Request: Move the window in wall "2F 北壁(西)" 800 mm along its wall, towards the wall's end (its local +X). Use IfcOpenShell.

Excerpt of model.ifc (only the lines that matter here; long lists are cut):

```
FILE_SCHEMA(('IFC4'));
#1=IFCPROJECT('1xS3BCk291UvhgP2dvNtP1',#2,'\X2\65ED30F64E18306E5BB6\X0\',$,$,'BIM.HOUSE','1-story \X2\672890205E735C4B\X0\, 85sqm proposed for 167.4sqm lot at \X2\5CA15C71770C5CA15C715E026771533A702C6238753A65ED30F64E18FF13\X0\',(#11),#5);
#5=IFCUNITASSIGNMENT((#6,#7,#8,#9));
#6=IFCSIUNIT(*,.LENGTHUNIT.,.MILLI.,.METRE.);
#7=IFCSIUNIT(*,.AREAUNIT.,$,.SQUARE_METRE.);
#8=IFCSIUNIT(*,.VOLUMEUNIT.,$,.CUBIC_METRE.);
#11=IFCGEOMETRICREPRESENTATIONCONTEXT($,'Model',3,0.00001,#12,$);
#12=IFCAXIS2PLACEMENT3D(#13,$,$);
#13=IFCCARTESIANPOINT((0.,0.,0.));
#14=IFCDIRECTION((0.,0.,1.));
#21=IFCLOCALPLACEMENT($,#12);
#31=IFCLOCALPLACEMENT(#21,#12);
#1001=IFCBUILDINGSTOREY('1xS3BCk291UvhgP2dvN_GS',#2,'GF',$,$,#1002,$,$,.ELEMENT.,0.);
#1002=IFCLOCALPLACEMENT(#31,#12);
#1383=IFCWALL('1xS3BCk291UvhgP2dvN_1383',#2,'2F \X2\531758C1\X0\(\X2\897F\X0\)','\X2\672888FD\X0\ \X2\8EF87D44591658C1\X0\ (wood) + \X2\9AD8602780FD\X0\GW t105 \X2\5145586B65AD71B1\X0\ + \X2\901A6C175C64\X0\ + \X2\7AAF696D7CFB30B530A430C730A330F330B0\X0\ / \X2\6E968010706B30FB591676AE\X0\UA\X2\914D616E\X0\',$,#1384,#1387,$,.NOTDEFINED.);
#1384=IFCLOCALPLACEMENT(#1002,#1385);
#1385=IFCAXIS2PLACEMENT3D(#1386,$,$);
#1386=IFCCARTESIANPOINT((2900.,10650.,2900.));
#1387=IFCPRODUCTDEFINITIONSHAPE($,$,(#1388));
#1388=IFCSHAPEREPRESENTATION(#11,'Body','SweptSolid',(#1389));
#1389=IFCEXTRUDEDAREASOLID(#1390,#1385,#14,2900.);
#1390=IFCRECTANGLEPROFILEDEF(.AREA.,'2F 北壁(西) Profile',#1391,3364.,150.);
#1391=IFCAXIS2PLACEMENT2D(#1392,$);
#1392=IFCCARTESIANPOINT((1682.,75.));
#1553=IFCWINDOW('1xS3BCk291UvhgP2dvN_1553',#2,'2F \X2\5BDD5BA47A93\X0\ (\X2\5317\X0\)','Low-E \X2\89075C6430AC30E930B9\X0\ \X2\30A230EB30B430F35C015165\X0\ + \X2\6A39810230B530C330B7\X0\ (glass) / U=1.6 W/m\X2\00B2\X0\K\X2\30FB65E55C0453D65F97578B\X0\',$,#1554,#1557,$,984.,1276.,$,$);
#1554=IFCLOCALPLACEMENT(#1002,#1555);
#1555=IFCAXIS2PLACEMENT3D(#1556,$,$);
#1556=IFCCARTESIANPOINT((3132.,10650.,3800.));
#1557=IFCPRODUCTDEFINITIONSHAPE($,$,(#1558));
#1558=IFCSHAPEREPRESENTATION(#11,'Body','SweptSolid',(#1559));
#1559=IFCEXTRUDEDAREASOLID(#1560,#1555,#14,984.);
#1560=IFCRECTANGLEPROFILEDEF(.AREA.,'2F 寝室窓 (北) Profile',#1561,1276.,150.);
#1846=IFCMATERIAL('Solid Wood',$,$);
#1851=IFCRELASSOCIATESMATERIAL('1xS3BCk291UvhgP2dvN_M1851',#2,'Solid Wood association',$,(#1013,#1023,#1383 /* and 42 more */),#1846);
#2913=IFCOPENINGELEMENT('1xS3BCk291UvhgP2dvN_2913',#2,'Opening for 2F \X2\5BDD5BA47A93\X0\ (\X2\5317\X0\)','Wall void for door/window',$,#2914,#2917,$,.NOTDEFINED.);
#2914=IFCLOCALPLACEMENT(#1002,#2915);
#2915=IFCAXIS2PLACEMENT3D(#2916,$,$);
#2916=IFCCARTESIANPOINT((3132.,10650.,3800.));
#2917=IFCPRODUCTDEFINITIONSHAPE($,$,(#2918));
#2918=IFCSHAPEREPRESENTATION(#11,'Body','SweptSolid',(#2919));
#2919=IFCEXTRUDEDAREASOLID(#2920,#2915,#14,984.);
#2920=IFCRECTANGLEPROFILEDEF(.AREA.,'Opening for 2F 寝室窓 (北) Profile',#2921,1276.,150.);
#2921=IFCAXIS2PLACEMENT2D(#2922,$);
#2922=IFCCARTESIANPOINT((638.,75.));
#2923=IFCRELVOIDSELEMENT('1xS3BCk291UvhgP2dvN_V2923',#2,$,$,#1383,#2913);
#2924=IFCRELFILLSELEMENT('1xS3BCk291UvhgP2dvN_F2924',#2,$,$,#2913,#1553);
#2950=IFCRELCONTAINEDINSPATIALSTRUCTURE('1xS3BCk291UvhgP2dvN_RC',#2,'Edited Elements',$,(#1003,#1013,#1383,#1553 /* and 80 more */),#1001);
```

```python
import ifcopenshell
import ifcopenshell.api.geometry
import ifcopenshell.util.placement
import ifcopenshell.util.unit

model = ifcopenshell.open("model.ifc")
unit_scale = ifcopenshell.util.unit.calculate_unit_scale(model)

window = model.by_guid("1xS3BCk291UvhgP2dvN_1553")
opening = window.FillsVoids[0].RelatingOpeningElement
wall = opening.VoidsElements[0].RelatingBuildingElement

wall_matrix = ifcopenshell.util.placement.get_local_placement(wall.ObjectPlacement)
shift = wall_matrix[:3, 0] * 0.8 / unit_scale
before = ifcopenshell.util.placement.get_local_placement(window.ObjectPlacement)[:3, 3].copy()

# The window is not placed relative to its opening, so move both.
for product in (opening, window):
    matrix = ifcopenshell.util.placement.get_local_placement(product.ObjectPlacement)
    matrix[:3, 3] += shift
    ifcopenshell.api.geometry.edit_object_placement(model, product=product, matrix=matrix, is_si=False)

after = ifcopenshell.util.placement.get_local_placement(window.ObjectPlacement)[:3, 3]
print("window moved by", (after - before).round(3) + 0.0)

model.write("model_edited.ifc")
```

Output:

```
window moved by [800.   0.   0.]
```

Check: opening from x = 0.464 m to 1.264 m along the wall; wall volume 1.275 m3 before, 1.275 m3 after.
